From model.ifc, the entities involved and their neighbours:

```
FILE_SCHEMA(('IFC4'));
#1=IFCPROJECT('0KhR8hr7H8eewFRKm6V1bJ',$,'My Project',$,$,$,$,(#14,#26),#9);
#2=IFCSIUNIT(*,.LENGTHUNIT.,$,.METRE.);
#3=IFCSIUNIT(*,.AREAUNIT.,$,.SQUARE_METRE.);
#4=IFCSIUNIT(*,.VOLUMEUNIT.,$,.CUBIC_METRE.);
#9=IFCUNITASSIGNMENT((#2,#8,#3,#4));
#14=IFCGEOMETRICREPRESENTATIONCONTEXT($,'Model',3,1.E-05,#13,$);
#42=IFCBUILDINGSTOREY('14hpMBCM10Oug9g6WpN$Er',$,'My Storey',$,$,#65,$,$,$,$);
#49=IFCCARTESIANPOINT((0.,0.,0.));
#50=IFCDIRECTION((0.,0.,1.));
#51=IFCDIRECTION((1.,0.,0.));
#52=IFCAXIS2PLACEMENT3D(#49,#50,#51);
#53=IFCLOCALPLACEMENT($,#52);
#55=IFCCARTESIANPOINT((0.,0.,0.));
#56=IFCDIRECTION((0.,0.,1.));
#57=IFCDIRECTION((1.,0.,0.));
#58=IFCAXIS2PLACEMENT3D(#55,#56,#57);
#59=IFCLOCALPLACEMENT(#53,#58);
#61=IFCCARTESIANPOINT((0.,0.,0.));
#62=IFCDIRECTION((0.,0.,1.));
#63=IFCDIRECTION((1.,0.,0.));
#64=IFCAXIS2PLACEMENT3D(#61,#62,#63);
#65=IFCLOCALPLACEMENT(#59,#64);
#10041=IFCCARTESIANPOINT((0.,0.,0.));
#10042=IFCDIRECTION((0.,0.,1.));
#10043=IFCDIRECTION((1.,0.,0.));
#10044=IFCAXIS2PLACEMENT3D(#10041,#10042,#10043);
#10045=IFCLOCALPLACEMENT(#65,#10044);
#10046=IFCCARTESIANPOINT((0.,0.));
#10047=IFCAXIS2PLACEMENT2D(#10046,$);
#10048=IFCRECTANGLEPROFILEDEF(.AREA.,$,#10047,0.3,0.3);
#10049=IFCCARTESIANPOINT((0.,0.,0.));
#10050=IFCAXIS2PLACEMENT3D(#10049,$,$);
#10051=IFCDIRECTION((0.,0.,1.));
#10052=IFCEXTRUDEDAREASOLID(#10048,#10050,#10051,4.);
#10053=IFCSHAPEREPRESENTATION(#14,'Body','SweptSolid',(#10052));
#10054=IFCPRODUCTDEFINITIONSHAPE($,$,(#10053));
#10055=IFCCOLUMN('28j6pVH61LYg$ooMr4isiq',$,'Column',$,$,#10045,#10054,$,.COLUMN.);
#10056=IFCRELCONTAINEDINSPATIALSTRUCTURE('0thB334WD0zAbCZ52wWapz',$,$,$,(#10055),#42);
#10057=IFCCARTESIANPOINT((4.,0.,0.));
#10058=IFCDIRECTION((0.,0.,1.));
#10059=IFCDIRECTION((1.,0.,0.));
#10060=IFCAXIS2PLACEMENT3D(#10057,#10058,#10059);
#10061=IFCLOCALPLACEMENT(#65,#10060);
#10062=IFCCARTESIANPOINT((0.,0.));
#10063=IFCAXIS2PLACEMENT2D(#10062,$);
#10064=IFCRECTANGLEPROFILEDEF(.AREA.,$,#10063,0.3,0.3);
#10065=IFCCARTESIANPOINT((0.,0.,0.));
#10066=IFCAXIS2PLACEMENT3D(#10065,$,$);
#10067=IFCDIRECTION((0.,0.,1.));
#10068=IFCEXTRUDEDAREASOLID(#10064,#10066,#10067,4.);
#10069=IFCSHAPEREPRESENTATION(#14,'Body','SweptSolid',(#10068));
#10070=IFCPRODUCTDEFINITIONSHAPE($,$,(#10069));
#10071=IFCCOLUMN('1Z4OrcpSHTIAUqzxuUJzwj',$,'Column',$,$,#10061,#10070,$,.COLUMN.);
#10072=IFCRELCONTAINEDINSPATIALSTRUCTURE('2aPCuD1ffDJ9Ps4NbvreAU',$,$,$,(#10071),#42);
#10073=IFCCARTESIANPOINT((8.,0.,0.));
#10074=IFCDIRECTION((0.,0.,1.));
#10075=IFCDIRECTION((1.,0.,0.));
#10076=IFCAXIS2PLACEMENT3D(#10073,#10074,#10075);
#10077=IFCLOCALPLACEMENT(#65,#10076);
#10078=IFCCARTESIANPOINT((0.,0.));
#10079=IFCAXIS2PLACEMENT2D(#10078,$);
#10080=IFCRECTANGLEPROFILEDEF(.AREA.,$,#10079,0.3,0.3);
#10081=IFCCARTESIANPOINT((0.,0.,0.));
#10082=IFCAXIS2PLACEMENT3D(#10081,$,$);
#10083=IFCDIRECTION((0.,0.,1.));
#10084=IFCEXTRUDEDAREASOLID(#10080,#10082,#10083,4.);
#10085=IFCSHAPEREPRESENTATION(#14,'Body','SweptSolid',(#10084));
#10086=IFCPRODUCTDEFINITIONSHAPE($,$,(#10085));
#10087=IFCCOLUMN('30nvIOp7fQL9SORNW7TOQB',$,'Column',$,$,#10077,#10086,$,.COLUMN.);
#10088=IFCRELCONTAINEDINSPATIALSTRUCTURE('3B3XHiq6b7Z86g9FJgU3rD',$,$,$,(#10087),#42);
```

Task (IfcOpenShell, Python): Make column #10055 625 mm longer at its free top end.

```python
import ifcopenshell
import ifcopenshell.util.unit

model = ifcopenshell.open("model.ifc")
unit_scale = ifcopenshell.util.unit.calculate_unit_scale(model)

member = model.by_guid("28j6pVH61LYg$ooMr4isiq")
change = 0.625 / unit_scale

# The extrusion runs towards the end named, so only its depth changes.
body = next(r for r in member.Representation.Representations if r.RepresentationIdentifier == "Body")
solid = body.Items[0]
old_length = solid.Depth
solid.Depth += change

print(f"length {old_length:g} -> {solid.Depth:g}")

model.write("model-out.ifc")
```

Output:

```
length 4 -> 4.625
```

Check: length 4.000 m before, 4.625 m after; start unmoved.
